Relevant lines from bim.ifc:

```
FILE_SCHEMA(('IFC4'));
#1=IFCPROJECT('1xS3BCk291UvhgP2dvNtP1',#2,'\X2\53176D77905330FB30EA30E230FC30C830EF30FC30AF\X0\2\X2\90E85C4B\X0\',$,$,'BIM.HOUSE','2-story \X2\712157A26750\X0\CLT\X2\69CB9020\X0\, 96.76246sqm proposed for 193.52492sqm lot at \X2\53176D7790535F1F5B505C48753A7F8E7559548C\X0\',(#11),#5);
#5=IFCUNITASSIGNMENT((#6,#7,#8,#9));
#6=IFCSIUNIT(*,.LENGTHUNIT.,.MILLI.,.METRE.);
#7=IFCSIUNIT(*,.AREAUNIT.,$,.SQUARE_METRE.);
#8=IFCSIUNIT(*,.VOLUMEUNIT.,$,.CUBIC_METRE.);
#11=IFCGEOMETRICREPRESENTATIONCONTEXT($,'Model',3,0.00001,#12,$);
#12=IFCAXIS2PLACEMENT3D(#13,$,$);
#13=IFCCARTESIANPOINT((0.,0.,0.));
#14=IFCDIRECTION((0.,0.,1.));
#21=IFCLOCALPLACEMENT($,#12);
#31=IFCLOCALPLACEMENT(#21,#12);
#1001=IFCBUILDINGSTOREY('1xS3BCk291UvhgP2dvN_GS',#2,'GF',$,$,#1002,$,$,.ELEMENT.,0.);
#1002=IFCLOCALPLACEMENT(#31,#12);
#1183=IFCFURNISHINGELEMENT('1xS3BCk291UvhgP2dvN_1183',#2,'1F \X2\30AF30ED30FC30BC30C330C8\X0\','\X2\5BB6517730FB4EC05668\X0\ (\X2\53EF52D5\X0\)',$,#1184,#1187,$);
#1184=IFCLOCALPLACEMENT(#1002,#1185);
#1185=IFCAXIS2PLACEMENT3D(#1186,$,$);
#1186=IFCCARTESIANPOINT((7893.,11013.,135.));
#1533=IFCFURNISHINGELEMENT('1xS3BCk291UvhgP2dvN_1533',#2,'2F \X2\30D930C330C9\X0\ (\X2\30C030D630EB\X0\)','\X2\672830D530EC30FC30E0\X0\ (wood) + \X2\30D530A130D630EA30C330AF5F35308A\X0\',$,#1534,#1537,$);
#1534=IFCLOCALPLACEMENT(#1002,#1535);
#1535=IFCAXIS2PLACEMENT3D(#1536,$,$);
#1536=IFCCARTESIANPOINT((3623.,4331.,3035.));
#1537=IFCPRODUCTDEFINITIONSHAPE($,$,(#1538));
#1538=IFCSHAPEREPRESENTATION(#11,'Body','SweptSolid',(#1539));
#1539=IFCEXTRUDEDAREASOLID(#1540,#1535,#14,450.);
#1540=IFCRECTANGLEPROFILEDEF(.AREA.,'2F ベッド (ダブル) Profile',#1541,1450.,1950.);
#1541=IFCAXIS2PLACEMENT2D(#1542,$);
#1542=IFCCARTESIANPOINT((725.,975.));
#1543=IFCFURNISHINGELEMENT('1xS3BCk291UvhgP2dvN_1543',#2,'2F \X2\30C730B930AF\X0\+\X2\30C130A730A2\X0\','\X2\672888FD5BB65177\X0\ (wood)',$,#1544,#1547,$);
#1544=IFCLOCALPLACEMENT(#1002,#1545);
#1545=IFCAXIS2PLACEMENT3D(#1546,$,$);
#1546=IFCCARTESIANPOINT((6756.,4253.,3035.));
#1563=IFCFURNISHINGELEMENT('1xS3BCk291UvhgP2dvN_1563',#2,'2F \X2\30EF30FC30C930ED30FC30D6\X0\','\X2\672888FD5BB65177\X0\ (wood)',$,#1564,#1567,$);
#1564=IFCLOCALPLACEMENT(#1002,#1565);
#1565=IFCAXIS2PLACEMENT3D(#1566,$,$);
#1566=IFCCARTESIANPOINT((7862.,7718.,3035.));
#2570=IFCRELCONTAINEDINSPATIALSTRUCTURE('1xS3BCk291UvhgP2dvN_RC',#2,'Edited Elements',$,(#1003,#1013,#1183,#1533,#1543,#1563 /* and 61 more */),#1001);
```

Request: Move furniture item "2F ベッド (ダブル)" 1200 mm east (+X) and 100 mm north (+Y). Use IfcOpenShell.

```python
import ifcopenshell
import ifcopenshell.api.geometry
import ifcopenshell.util.placement

model = ifcopenshell.open("bim.ifc")

item = model.by_guid("1xS3BCk291UvhgP2dvN_1533")
matrix = ifcopenshell.util.placement.get_local_placement(item.ObjectPlacement)
matrix[0, 3] += 1200.0
matrix[1, 3] += 100.0
ifcopenshell.api.geometry.edit_object_placement(model, product=item, matrix=matrix, is_si=False)

print(ifcopenshell.util.placement.get_local_placement(item.ObjectPlacement).round(3) + 0.0)

model.write("bim_updated.ifc")
```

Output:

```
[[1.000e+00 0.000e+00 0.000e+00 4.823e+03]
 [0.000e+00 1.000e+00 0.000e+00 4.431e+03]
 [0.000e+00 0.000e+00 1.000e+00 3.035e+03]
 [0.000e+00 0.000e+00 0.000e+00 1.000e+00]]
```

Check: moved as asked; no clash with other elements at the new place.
